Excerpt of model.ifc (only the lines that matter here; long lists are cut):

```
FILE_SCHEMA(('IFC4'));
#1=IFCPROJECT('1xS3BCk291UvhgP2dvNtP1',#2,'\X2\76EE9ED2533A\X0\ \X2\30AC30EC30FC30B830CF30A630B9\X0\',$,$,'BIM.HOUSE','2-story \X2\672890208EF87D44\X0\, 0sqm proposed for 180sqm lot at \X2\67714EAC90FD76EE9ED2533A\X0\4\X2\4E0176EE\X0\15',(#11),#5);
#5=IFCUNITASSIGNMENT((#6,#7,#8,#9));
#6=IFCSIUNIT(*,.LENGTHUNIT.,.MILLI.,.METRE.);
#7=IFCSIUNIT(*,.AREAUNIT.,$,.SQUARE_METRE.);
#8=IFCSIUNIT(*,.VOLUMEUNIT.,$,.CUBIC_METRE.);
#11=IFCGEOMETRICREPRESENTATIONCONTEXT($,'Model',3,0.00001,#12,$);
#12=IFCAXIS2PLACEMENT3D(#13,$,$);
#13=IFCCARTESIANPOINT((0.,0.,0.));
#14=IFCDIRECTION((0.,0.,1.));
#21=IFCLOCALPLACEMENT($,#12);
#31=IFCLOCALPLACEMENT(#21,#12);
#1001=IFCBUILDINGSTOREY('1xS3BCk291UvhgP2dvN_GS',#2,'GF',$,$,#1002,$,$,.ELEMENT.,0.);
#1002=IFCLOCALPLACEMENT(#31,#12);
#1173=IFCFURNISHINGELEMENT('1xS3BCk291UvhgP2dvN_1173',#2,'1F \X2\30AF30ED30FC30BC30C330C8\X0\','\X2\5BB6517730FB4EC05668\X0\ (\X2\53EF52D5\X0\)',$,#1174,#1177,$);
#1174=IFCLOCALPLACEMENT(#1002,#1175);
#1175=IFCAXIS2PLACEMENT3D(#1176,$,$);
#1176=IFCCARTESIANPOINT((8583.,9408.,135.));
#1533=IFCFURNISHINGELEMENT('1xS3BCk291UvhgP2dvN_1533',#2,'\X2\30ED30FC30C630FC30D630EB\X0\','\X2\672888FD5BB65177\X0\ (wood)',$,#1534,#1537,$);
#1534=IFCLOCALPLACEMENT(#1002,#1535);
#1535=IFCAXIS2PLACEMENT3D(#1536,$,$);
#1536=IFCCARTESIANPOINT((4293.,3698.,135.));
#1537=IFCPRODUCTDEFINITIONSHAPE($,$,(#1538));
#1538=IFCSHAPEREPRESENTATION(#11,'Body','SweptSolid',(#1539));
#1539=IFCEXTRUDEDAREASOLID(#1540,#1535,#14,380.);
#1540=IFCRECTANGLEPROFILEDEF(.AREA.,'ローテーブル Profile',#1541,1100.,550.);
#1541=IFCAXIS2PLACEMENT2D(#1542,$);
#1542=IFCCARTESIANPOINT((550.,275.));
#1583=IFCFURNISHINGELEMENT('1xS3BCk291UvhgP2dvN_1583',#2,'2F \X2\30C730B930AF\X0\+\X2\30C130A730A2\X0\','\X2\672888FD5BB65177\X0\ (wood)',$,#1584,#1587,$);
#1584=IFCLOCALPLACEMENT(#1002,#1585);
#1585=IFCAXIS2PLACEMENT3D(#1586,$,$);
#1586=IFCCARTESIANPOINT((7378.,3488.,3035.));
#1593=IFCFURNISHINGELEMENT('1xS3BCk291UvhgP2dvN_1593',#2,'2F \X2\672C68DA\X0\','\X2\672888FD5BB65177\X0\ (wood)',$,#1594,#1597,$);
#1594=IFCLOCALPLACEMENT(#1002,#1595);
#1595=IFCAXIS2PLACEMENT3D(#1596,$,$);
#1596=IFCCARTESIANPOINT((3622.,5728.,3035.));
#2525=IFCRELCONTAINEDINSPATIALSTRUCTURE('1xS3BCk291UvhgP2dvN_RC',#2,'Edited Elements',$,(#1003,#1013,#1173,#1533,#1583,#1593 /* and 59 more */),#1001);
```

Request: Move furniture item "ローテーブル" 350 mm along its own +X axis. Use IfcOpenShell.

```python
import ifcopenshell
import ifcopenshell.api.geometry
import ifcopenshell.util.placement
import ifcopenshell.util.unit

model = ifcopenshell.open("model.ifc")
unit_scale = ifcopenshell.util.unit.calculate_unit_scale(model)

item = model.by_guid("1xS3BCk291UvhgP2dvN_1533")
matrix = ifcopenshell.util.placement.get_local_placement(item.ObjectPlacement)
matrix[:3, 3] += matrix[:3, 0] * 0.35 / unit_scale
ifcopenshell.api.geometry.edit_object_placement(model, product=item, matrix=matrix, is_si=False)

print(ifcopenshell.util.placement.get_local_placement(item.ObjectPlacement).round(3) + 0.0)

model.write("model_updated.ifc")
```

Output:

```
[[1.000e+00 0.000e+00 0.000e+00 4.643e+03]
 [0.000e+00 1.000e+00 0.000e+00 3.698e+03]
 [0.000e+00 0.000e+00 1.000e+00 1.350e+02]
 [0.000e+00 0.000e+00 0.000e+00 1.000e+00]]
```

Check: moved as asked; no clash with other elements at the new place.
